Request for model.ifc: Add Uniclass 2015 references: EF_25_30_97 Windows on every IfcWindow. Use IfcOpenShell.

First a look at what the model holds.

```python
import ifcopenshell

model = ifcopenshell.open("model.ifc")
print(model.schema)
print("classifications:", [c.Name for c in model.by_type("IfcClassification")])
for ifc_class in ("IfcDoor", "IfcRoof", "IfcStair", "IfcWall", "IfcWindow"):
    print(ifc_class, len(model.by_type(ifc_class)))
```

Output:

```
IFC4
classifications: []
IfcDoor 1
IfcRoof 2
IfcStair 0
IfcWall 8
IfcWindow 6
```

```python
import ifcopenshell
import ifcopenshell.api.classification

model = ifcopenshell.open("model.ifc")

system = ifcopenshell.api.classification.add_classification(model, classification="Uniclass 2015")

codes = {
    "IfcWindow": ("EF_25_30_97", "Windows"),
}
for ifc_class, (code, name) in codes.items():
    products = model.by_type(ifc_class)
    ifcopenshell.api.classification.add_reference(
        model, products=products, classification=system, identification=code, name=name
    )
    print(code, len(products))

model.write("model_rev.ifc")
```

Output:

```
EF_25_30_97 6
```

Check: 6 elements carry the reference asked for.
